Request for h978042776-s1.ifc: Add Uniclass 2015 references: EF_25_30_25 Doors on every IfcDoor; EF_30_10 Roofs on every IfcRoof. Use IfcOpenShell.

First a look at what the model holds.

```python
import ifcopenshell

model = ifcopenshell.open("h978042776-s1.ifc")
print(model.schema)
print("classifications:", [c.Name for c in model.by_type("IfcClassification")])
for ifc_class in ("IfcDoor", "IfcRoof", "IfcStair", "IfcWall", "IfcWindow"):
    print(ifc_class, len(model.by_type(ifc_class)))
```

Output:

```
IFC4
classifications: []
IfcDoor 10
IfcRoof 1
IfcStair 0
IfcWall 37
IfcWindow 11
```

```python
import ifcopenshell
import ifcopenshell.api.classification

model = ifcopenshell.open("h978042776-s1.ifc")

system = ifcopenshell.api.classification.add_classification(model, classification="Uniclass 2015")

codes = {
    "IfcDoor": ("EF_25_30_25", "Doors"),
    "IfcRoof": ("EF_30_10", "Roofs"),
}
for ifc_class, (code, name) in codes.items():
    products = model.by_type(ifc_class)
    ifcopenshell.api.classification.add_reference(
        model, products=products, classification=system, identification=code, name=name
    )
    print(code, len(products))

model.write("h978042776-s1_v2.ifc")
```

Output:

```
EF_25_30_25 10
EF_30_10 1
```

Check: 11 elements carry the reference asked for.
